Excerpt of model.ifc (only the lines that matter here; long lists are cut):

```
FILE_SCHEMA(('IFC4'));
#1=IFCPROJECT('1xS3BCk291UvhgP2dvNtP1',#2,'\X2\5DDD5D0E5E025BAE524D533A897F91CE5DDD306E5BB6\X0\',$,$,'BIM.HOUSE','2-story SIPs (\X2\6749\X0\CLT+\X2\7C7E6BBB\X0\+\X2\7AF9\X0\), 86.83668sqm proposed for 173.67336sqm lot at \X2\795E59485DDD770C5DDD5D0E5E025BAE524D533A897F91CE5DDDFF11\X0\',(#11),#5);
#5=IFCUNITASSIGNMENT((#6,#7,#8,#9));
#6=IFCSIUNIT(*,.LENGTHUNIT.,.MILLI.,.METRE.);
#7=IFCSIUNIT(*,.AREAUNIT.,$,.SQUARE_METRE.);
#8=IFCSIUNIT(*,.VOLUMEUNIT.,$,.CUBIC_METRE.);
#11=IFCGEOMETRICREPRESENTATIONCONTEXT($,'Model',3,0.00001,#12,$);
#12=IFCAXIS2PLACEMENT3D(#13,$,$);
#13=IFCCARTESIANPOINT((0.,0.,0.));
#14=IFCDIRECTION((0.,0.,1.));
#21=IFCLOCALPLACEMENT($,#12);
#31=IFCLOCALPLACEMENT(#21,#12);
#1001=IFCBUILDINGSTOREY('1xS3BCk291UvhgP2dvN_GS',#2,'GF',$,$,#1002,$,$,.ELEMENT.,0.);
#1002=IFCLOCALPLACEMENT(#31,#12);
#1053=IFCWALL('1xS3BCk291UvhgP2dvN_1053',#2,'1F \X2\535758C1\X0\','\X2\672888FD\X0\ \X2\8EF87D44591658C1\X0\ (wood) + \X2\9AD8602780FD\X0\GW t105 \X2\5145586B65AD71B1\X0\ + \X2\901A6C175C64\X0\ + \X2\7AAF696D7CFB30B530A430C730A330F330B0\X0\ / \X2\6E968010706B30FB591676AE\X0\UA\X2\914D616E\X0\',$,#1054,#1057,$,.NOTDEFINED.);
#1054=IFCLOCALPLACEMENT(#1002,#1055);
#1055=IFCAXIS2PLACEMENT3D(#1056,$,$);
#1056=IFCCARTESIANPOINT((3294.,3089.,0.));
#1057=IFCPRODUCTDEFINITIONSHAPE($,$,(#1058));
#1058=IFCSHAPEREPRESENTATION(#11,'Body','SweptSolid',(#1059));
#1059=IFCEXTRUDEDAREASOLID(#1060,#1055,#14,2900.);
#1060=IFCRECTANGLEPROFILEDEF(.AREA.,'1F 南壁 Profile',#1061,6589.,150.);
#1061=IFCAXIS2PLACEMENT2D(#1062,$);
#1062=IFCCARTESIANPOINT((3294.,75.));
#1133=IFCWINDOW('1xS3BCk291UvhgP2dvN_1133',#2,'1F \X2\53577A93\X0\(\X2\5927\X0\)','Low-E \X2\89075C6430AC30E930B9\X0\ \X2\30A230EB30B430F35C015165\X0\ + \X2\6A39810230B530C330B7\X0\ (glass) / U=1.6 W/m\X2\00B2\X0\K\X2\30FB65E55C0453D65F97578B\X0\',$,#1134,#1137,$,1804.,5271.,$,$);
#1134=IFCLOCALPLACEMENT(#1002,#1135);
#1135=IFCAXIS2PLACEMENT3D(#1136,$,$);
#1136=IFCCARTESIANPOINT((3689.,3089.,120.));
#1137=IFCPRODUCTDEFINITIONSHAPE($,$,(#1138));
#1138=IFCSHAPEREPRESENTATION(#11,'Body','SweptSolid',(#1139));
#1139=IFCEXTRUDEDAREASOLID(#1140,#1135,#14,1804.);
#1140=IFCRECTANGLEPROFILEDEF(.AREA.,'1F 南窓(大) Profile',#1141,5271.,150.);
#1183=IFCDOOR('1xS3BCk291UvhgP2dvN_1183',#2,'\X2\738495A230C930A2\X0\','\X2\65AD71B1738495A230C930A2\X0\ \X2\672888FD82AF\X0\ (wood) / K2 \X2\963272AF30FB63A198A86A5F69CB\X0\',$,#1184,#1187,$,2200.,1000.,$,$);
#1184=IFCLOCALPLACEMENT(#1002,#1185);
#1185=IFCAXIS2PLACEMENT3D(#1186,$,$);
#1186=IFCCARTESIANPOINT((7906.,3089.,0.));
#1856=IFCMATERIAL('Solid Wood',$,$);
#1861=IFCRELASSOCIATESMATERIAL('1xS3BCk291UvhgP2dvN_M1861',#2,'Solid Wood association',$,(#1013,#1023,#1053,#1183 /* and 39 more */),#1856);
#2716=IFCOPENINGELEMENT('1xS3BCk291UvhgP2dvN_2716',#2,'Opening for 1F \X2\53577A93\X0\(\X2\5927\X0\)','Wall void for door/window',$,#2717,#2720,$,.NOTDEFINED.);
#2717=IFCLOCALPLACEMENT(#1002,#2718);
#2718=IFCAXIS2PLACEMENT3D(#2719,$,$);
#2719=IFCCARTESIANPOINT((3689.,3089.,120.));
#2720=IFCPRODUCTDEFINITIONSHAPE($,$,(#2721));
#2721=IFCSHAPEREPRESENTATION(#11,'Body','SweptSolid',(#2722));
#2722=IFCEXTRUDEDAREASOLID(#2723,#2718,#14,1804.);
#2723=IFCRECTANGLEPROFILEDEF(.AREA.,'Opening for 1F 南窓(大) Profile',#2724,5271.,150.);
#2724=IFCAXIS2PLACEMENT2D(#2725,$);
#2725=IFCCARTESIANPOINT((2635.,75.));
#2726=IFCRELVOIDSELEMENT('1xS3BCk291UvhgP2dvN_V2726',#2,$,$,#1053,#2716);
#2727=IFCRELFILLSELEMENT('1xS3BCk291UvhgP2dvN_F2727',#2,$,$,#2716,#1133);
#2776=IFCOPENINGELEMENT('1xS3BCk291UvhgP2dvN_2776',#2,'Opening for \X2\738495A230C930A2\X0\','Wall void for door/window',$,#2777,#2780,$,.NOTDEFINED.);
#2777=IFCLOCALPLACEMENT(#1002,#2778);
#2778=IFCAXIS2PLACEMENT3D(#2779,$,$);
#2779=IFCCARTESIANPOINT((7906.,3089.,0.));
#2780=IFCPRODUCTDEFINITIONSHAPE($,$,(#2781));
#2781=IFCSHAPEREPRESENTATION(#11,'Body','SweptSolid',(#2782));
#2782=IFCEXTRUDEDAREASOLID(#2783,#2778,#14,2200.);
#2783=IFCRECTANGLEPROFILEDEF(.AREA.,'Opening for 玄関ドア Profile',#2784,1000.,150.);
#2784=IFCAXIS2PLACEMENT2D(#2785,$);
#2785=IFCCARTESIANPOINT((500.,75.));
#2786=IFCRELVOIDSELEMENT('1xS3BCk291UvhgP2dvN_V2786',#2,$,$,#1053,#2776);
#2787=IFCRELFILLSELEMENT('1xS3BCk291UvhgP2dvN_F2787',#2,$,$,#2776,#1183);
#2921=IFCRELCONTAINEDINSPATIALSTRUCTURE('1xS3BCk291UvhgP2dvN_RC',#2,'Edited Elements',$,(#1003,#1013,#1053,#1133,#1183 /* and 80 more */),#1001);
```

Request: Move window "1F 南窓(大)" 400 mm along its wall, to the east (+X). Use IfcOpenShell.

```python
import ifcopenshell
import ifcopenshell.api.geometry
import ifcopenshell.util.placement
import ifcopenshell.util.unit

model = ifcopenshell.open("model.ifc")
unit_scale = ifcopenshell.util.unit.calculate_unit_scale(model)

window = model.by_guid("1xS3BCk291UvhgP2dvN_1133")
opening = window.FillsVoids[0].RelatingOpeningElement
wall = opening.VoidsElements[0].RelatingBuildingElement

wall_matrix = ifcopenshell.util.placement.get_local_placement(wall.ObjectPlacement)
shift = wall_matrix[:3, 0] * 0.4 / unit_scale
before = ifcopenshell.util.placement.get_local_placement(window.ObjectPlacement)[:3, 3].copy()

# The window is not placed relative to its opening, so move both.
for product in (opening, window):
    matrix = ifcopenshell.util.placement.get_local_placement(product.ObjectPlacement)
    matrix[:3, 3] += shift
    ifcopenshell.api.geometry.edit_object_placement(model, product=product, matrix=matrix, is_si=False)

after = ifcopenshell.util.placement.get_local_placement(window.ObjectPlacement)[:3, 3]
print("window moved by", (after - before).round(3) + 0.0)

model.write("model_v2.ifc")
```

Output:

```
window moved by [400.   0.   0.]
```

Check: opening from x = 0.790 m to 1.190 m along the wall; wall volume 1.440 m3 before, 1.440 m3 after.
